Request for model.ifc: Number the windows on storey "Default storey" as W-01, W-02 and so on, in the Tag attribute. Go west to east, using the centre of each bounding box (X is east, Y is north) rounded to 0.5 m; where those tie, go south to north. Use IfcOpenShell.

First a look at what the model holds.

```python
import ifcopenshell
import ifcopenshell.util.element
import ifcopenshell.util.placement

model = ifcopenshell.open("model.ifc")
print(model.schema)
storey = next(s for s in model.by_type("IfcBuildingStorey") if s.Name == "Default storey")
windows = [e for e in ifcopenshell.util.element.get_decomposition(storey) if e.is_a("IfcWindow")]
for e in sorted(windows, key=lambda e: e.id()):
    origin = ifcopenshell.util.placement.get_local_placement(e.ObjectPlacement)[:3, 3]
    print(e.id(), e.Tag, e.Name, origin.round(2) + 0.0, sep=" | ")
```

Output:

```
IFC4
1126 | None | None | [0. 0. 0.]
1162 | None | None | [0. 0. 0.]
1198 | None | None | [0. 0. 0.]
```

```python
import ifcopenshell
import ifcopenshell.geom
import ifcopenshell.util.element
import ifcopenshell.util.shape

model = ifcopenshell.open("model.ifc")
settings = ifcopenshell.geom.settings()
settings.set("use-world-coords", True)


def centre(element):
    shape = ifcopenshell.geom.create_shape(settings, element)
    return ifcopenshell.util.shape.get_bbox_centroid(shape.geometry)


storey = next(s for s in model.by_type("IfcBuildingStorey") if s.Name == "Default storey")
windows = [e for e in ifcopenshell.util.element.get_decomposition(storey) if e.is_a("IfcWindow")]

# Insertion points can sit at a corner or the storey origin, so sort by the geometry (in metres).
centres = {e: centre(e) for e in windows}
windows.sort(key=lambda e: (round(centres[e][0] / 0.5), centres[e][1]))

for i, e in enumerate(windows, start=1):
    number = f"W-{i:02d}"
    e.Tag = number
    print(e.id(), number)

model.write("model_edited.ifc")
```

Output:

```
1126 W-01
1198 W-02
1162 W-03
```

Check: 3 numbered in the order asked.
